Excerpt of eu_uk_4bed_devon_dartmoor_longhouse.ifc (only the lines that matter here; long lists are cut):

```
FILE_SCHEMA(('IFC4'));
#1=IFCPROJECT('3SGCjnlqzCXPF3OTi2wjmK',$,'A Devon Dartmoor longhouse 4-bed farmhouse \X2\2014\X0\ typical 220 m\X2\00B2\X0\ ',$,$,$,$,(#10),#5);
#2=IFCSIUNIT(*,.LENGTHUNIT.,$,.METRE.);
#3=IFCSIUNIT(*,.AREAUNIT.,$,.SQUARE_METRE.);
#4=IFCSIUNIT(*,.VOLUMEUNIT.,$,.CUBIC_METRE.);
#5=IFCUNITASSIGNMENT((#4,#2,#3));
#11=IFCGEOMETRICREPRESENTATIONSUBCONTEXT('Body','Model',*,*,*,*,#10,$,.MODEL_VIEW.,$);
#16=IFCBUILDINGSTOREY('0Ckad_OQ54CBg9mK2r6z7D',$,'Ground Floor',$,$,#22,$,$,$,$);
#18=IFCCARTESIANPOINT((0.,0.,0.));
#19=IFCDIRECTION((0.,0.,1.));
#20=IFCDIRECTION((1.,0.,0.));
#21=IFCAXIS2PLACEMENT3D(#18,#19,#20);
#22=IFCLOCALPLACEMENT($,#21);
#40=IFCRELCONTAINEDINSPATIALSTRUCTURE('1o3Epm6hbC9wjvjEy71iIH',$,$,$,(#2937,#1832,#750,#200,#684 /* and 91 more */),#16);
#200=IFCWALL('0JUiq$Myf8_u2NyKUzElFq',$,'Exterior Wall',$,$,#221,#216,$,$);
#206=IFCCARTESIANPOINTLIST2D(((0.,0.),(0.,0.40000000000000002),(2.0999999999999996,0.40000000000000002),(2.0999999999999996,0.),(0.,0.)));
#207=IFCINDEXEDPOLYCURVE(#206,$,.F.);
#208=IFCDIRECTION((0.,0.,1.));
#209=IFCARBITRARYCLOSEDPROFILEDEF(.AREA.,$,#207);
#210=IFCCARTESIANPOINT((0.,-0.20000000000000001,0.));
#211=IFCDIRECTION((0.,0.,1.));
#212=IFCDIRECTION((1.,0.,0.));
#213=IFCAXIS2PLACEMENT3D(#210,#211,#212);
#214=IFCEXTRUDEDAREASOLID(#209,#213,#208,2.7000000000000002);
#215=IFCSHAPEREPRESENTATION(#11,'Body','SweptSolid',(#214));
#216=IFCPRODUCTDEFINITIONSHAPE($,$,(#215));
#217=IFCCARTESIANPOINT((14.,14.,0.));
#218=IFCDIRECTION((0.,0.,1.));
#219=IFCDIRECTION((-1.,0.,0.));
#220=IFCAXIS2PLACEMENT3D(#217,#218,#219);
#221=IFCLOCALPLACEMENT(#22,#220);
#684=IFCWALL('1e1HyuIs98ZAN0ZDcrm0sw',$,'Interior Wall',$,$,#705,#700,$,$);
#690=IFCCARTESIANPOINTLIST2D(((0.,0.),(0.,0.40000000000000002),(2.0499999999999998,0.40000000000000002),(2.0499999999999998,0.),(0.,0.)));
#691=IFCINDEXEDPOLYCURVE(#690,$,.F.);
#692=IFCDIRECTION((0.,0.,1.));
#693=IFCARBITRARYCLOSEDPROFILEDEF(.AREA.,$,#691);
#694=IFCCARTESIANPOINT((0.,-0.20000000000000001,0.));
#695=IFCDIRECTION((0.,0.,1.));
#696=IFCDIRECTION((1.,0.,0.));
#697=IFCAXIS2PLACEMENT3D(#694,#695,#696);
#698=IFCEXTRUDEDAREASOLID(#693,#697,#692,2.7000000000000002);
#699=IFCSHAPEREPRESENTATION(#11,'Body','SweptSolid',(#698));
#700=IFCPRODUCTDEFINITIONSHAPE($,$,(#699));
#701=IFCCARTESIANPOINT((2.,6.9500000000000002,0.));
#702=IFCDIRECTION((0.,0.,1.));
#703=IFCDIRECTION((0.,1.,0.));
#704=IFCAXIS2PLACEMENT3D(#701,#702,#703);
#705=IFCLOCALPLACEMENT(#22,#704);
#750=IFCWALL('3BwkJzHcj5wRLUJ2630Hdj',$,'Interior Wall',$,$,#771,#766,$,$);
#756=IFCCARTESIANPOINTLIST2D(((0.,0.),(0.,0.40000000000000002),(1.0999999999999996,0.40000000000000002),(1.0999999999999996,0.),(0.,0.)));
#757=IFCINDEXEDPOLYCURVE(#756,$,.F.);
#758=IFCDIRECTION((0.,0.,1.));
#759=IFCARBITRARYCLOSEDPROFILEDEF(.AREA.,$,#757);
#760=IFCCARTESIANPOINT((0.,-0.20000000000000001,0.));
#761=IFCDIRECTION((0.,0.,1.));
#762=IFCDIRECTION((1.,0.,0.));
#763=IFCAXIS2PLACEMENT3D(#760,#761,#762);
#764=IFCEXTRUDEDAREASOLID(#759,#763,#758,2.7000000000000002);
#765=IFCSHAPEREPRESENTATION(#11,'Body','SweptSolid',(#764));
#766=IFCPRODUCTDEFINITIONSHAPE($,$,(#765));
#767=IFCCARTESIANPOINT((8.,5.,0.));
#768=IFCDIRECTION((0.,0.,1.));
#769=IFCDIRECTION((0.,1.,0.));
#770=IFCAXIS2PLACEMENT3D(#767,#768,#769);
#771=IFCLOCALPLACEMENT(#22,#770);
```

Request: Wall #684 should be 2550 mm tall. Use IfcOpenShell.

```python
import ifcopenshell
import ifcopenshell.geom
import ifcopenshell.util.representation
import ifcopenshell.util.shape

model = ifcopenshell.open("eu_uk_4bed_devon_dartmoor_longhouse.ifc")
settings = ifcopenshell.geom.settings()


def volume(element):
    """Net volume in cubic metres, openings subtracted."""
    shape = ifcopenshell.geom.create_shape(settings, element)
    return ifcopenshell.util.shape.get_volume(shape.geometry)


wall = model.by_guid("1e1HyuIs98ZAN0ZDcrm0sw")
before = volume(wall)

body = ifcopenshell.util.representation.get_representation(wall, "Model", "Body")
solid = body.Items[0]
old_height = solid.Depth
solid.Depth = 2.55
after = volume(wall)

print(f"height {old_height:g} -> {solid.Depth:g}, volume {before:.3f} -> {after:.3f} m3")

model.write("eu_uk_4bed_devon_dartmoor_longhouse_updated.ifc")
```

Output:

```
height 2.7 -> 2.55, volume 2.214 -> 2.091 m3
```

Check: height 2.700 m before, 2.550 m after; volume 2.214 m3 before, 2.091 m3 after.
